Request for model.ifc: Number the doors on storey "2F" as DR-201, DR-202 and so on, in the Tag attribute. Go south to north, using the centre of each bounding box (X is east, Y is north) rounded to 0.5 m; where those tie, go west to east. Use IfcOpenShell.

First a look at what the model holds.

```python
import ifcopenshell
import ifcopenshell.util.element
import ifcopenshell.util.placement

model = ifcopenshell.open("model.ifc")
print(model.schema)
storey = next(s for s in model.by_type("IfcBuildingStorey") if s.Name == "2F")
doors = [e for e in ifcopenshell.util.element.get_decomposition(storey) if e.is_a("IfcDoor")]
for e in sorted(doors, key=lambda e: e.id()):
    origin = ifcopenshell.util.placement.get_local_placement(e.ObjectPlacement)[:3, 3]
    print(e.id(), e.Tag, e.Name, origin.round(2) + 0.0, sep=" | ")
```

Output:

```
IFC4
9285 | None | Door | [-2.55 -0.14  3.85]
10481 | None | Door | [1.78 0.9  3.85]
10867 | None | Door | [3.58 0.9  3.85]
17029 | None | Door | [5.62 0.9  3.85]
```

```python
import ifcopenshell
import ifcopenshell.geom
import ifcopenshell.util.element
import ifcopenshell.util.shape

model = ifcopenshell.open("model.ifc")
settings = ifcopenshell.geom.settings()
settings.set("use-world-coords", True)


def centre(element):
    shape = ifcopenshell.geom.create_shape(settings, element)
    return ifcopenshell.util.shape.get_bbox_centroid(shape.geometry)


storey = next(s for s in model.by_type("IfcBuildingStorey") if s.Name == "2F")
doors = [e for e in ifcopenshell.util.element.get_decomposition(storey) if e.is_a("IfcDoor")]

# Insertion points can sit at a corner or the storey origin, so sort by the geometry (in metres).
centres = {e: centre(e) for e in doors}
doors.sort(key=lambda e: (round(centres[e][1] / 0.5), centres[e][0]))

for i, e in enumerate(doors, start=1):
    number = f"DR-2{i:02d}"
    e.Tag = number
    print(e.id(), number)

model.write("model-out.ifc")
```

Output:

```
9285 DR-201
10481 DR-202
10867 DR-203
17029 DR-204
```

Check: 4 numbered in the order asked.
